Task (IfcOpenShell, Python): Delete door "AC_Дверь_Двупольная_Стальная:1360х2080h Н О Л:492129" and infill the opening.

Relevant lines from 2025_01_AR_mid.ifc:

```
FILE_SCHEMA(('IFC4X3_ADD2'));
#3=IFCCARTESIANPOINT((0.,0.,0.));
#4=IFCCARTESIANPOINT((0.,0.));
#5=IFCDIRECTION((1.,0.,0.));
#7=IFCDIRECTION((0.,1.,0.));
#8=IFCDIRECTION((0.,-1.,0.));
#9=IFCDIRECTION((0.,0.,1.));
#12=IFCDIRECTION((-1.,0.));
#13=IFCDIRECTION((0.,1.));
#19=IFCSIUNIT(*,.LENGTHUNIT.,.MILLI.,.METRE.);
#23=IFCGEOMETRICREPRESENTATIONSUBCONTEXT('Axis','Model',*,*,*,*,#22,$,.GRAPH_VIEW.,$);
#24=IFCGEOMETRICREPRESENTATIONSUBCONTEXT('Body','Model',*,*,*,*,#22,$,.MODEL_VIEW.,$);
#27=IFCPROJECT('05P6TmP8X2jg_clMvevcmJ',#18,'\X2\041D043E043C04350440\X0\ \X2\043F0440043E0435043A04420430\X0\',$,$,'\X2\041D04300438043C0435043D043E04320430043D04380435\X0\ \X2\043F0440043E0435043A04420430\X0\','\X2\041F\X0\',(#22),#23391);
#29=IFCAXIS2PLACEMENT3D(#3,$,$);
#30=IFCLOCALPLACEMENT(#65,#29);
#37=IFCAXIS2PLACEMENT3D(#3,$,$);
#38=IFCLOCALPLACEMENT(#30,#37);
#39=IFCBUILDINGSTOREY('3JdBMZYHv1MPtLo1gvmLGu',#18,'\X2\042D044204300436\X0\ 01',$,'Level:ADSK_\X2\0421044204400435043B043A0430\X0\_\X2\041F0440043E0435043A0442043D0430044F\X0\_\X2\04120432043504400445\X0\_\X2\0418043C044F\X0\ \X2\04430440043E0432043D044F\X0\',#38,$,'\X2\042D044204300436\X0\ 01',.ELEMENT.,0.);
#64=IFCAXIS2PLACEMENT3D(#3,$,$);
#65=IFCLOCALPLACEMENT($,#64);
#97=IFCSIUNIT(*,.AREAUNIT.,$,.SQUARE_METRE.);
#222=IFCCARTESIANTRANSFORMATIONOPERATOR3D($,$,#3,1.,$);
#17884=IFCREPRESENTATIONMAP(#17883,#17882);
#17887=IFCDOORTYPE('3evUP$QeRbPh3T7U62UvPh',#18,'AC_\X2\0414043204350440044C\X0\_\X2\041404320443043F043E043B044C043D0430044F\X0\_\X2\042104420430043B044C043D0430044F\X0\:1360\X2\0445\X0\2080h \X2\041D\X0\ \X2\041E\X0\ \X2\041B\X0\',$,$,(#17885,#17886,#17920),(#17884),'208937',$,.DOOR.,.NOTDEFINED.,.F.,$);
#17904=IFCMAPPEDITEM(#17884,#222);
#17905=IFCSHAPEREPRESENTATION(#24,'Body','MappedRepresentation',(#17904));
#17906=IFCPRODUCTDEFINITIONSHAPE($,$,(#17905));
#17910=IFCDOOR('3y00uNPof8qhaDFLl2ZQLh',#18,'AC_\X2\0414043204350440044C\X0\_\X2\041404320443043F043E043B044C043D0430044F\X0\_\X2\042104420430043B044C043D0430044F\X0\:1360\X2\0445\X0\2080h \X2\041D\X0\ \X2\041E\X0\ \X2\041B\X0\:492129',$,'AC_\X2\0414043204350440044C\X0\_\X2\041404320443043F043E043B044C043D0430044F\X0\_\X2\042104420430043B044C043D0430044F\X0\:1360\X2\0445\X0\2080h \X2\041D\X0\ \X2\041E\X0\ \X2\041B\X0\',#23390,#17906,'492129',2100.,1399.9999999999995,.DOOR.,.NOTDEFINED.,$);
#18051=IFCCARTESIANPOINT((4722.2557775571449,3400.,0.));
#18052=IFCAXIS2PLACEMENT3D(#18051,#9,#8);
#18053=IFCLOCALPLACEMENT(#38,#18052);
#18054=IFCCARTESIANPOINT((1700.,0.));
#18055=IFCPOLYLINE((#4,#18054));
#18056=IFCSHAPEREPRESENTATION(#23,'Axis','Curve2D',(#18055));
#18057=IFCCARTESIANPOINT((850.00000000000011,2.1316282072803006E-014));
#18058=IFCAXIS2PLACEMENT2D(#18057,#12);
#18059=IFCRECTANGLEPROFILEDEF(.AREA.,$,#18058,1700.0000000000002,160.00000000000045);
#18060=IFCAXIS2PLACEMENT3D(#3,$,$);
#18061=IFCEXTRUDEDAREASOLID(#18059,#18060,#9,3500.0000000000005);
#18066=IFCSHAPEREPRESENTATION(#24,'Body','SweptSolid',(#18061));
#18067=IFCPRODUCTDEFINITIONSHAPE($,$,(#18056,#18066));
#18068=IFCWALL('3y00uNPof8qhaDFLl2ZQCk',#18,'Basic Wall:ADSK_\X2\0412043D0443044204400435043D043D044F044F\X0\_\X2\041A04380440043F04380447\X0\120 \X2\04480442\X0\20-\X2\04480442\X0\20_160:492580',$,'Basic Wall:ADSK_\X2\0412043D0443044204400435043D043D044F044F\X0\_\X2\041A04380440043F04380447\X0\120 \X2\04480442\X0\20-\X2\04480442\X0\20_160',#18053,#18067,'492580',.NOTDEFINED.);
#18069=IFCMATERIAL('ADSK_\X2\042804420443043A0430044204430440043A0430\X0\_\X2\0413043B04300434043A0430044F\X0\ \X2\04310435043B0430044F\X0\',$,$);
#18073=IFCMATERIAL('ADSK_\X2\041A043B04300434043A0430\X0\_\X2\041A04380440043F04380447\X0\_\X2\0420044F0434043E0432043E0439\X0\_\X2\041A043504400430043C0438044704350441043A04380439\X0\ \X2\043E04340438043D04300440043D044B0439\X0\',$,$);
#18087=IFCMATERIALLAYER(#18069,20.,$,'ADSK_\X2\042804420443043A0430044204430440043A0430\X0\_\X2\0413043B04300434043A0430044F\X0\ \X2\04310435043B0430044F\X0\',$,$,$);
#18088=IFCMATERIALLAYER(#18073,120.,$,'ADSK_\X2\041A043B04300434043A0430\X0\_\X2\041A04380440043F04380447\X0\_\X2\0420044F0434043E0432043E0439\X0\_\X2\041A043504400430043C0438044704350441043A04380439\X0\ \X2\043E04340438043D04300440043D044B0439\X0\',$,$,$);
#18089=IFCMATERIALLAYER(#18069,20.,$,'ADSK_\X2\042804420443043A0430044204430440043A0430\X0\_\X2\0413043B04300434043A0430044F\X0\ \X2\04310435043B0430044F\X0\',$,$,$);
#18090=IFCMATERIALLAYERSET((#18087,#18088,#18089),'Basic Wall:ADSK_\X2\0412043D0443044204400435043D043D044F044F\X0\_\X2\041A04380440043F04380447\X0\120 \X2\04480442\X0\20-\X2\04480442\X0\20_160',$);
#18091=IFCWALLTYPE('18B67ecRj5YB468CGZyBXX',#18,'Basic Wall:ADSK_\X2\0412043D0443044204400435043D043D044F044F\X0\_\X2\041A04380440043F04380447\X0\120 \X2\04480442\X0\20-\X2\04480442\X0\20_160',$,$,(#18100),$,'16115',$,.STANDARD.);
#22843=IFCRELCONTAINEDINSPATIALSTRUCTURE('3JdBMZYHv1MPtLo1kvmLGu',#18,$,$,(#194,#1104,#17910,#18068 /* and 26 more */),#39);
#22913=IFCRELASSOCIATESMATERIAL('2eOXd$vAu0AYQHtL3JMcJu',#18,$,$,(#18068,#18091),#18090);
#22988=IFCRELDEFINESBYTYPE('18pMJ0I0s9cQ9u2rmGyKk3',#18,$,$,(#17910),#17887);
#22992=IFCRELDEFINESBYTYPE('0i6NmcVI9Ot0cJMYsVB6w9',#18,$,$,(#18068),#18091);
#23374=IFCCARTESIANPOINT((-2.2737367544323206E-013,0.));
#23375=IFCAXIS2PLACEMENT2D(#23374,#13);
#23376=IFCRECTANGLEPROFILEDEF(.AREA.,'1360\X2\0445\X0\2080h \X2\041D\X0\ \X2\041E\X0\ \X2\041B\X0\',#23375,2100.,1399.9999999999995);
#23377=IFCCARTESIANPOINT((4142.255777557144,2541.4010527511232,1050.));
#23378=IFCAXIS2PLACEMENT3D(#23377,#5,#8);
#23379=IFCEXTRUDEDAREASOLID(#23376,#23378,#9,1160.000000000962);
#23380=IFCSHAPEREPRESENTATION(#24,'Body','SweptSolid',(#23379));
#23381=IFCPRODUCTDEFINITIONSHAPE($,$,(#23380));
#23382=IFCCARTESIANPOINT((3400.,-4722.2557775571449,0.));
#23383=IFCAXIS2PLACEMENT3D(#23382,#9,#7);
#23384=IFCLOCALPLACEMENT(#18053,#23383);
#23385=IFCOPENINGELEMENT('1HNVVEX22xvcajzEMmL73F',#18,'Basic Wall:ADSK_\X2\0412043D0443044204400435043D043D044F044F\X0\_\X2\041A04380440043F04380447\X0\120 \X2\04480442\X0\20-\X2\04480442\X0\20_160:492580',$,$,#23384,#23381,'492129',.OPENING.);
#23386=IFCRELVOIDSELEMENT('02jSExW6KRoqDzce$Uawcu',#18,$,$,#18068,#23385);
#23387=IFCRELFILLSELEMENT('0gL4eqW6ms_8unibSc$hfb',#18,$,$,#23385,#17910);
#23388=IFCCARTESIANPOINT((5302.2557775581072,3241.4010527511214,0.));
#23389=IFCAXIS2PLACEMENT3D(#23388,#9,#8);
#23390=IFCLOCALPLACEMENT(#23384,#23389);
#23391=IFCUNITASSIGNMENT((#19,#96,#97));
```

```python
import ifcopenshell
import ifcopenshell.api.feature
import ifcopenshell.api.root
import ifcopenshell.geom
import ifcopenshell.util.shape

model = ifcopenshell.open("2025_01_AR_mid.ifc")
settings = ifcopenshell.geom.settings()


def volume(element):
    """Net volume in cubic metres, openings subtracted."""
    shape = ifcopenshell.geom.create_shape(settings, element)
    return ifcopenshell.util.shape.get_volume(shape.geometry)


door = model.by_guid("3y00uNPof8qhaDFLl2ZQLh")
opening = door.FillsVoids[0].RelatingOpeningElement
wall = opening.VoidsElements[0].RelatingBuildingElement
before = volume(wall)

ifcopenshell.api.root.remove_product(model, product=door)
ifcopenshell.api.feature.remove_feature(model, feature=opening)

after = volume(wall)

print(f"wall volume {before:.3f} -> {after:.3f} m3")

model.write("2025_01_AR_mid-out.ifc")
```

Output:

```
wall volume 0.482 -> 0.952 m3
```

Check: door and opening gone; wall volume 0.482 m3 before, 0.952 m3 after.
